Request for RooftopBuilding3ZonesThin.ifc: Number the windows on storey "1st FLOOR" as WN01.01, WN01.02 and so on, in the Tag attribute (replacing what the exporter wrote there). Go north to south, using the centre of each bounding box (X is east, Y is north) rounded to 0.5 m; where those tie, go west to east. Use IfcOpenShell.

First a look at what the model holds.

```python
import ifcopenshell
import ifcopenshell.util.element
import ifcopenshell.util.placement

model = ifcopenshell.open("RooftopBuilding3ZonesThin.ifc")
print(model.schema)
storey = next(s for s in model.by_type("IfcBuildingStorey") if s.Name == "1st FLOOR")
windows = [e for e in ifcopenshell.util.element.get_decomposition(storey) if e.is_a("IfcWindow")]
for e in sorted(windows, key=lambda e: e.id()):
    origin = ifcopenshell.util.placement.get_local_placement(e.ObjectPlacement)[:3, 3]
    print(e.id(), e.Tag, e.Name, origin.round(2) + 0.0, sep=" | ")
```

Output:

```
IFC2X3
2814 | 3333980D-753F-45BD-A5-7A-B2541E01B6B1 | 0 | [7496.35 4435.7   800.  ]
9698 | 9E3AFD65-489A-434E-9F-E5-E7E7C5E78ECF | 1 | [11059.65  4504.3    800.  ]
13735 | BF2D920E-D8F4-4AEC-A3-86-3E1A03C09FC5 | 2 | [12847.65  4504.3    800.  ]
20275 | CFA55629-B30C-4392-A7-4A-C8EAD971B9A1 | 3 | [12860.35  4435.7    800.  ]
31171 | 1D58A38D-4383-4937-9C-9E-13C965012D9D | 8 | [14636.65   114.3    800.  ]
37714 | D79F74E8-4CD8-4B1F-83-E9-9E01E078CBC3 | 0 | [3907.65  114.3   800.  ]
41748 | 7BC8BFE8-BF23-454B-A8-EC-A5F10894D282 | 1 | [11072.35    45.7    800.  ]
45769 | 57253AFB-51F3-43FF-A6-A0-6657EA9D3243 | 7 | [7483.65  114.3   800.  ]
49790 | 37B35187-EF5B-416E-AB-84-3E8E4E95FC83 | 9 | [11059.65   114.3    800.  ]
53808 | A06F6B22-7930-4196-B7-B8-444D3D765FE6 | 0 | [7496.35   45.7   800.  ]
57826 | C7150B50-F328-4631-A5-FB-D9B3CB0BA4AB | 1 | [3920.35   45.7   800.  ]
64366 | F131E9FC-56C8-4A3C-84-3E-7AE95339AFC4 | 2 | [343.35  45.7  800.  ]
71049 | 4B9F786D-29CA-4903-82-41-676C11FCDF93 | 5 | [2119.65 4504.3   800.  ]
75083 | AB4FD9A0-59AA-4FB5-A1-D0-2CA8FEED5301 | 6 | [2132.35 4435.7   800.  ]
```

```python
import ifcopenshell
import ifcopenshell.geom
import ifcopenshell.util.element
import ifcopenshell.util.shape

model = ifcopenshell.open("RooftopBuilding3ZonesThin.ifc")
settings = ifcopenshell.geom.settings()
settings.set("use-world-coords", True)


def centre(element):
    shape = ifcopenshell.geom.create_shape(settings, element)
    return ifcopenshell.util.shape.get_bbox_centroid(shape.geometry)


storey = next(s for s in model.by_type("IfcBuildingStorey") if s.Name == "1st FLOOR")
windows = [e for e in ifcopenshell.util.element.get_decomposition(storey) if e.is_a("IfcWindow")]

# Insertion points can sit at a corner or the storey origin, so sort by the geometry (in metres).
centres = {e: centre(e) for e in windows}
windows.sort(key=lambda e: (-round(centres[e][1] / 0.5), centres[e][0]))

for i, e in enumerate(windows, start=1):
    number = f"WN01.{i:02d}"
    e.Tag = number
    print(e.id(), number)

model.write("RooftopBuilding3ZonesThin_updated.ifc")
```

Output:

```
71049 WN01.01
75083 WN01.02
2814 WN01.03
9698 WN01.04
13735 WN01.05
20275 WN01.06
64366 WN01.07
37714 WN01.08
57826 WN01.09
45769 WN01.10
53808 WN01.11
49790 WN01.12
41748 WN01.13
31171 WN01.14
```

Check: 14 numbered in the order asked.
